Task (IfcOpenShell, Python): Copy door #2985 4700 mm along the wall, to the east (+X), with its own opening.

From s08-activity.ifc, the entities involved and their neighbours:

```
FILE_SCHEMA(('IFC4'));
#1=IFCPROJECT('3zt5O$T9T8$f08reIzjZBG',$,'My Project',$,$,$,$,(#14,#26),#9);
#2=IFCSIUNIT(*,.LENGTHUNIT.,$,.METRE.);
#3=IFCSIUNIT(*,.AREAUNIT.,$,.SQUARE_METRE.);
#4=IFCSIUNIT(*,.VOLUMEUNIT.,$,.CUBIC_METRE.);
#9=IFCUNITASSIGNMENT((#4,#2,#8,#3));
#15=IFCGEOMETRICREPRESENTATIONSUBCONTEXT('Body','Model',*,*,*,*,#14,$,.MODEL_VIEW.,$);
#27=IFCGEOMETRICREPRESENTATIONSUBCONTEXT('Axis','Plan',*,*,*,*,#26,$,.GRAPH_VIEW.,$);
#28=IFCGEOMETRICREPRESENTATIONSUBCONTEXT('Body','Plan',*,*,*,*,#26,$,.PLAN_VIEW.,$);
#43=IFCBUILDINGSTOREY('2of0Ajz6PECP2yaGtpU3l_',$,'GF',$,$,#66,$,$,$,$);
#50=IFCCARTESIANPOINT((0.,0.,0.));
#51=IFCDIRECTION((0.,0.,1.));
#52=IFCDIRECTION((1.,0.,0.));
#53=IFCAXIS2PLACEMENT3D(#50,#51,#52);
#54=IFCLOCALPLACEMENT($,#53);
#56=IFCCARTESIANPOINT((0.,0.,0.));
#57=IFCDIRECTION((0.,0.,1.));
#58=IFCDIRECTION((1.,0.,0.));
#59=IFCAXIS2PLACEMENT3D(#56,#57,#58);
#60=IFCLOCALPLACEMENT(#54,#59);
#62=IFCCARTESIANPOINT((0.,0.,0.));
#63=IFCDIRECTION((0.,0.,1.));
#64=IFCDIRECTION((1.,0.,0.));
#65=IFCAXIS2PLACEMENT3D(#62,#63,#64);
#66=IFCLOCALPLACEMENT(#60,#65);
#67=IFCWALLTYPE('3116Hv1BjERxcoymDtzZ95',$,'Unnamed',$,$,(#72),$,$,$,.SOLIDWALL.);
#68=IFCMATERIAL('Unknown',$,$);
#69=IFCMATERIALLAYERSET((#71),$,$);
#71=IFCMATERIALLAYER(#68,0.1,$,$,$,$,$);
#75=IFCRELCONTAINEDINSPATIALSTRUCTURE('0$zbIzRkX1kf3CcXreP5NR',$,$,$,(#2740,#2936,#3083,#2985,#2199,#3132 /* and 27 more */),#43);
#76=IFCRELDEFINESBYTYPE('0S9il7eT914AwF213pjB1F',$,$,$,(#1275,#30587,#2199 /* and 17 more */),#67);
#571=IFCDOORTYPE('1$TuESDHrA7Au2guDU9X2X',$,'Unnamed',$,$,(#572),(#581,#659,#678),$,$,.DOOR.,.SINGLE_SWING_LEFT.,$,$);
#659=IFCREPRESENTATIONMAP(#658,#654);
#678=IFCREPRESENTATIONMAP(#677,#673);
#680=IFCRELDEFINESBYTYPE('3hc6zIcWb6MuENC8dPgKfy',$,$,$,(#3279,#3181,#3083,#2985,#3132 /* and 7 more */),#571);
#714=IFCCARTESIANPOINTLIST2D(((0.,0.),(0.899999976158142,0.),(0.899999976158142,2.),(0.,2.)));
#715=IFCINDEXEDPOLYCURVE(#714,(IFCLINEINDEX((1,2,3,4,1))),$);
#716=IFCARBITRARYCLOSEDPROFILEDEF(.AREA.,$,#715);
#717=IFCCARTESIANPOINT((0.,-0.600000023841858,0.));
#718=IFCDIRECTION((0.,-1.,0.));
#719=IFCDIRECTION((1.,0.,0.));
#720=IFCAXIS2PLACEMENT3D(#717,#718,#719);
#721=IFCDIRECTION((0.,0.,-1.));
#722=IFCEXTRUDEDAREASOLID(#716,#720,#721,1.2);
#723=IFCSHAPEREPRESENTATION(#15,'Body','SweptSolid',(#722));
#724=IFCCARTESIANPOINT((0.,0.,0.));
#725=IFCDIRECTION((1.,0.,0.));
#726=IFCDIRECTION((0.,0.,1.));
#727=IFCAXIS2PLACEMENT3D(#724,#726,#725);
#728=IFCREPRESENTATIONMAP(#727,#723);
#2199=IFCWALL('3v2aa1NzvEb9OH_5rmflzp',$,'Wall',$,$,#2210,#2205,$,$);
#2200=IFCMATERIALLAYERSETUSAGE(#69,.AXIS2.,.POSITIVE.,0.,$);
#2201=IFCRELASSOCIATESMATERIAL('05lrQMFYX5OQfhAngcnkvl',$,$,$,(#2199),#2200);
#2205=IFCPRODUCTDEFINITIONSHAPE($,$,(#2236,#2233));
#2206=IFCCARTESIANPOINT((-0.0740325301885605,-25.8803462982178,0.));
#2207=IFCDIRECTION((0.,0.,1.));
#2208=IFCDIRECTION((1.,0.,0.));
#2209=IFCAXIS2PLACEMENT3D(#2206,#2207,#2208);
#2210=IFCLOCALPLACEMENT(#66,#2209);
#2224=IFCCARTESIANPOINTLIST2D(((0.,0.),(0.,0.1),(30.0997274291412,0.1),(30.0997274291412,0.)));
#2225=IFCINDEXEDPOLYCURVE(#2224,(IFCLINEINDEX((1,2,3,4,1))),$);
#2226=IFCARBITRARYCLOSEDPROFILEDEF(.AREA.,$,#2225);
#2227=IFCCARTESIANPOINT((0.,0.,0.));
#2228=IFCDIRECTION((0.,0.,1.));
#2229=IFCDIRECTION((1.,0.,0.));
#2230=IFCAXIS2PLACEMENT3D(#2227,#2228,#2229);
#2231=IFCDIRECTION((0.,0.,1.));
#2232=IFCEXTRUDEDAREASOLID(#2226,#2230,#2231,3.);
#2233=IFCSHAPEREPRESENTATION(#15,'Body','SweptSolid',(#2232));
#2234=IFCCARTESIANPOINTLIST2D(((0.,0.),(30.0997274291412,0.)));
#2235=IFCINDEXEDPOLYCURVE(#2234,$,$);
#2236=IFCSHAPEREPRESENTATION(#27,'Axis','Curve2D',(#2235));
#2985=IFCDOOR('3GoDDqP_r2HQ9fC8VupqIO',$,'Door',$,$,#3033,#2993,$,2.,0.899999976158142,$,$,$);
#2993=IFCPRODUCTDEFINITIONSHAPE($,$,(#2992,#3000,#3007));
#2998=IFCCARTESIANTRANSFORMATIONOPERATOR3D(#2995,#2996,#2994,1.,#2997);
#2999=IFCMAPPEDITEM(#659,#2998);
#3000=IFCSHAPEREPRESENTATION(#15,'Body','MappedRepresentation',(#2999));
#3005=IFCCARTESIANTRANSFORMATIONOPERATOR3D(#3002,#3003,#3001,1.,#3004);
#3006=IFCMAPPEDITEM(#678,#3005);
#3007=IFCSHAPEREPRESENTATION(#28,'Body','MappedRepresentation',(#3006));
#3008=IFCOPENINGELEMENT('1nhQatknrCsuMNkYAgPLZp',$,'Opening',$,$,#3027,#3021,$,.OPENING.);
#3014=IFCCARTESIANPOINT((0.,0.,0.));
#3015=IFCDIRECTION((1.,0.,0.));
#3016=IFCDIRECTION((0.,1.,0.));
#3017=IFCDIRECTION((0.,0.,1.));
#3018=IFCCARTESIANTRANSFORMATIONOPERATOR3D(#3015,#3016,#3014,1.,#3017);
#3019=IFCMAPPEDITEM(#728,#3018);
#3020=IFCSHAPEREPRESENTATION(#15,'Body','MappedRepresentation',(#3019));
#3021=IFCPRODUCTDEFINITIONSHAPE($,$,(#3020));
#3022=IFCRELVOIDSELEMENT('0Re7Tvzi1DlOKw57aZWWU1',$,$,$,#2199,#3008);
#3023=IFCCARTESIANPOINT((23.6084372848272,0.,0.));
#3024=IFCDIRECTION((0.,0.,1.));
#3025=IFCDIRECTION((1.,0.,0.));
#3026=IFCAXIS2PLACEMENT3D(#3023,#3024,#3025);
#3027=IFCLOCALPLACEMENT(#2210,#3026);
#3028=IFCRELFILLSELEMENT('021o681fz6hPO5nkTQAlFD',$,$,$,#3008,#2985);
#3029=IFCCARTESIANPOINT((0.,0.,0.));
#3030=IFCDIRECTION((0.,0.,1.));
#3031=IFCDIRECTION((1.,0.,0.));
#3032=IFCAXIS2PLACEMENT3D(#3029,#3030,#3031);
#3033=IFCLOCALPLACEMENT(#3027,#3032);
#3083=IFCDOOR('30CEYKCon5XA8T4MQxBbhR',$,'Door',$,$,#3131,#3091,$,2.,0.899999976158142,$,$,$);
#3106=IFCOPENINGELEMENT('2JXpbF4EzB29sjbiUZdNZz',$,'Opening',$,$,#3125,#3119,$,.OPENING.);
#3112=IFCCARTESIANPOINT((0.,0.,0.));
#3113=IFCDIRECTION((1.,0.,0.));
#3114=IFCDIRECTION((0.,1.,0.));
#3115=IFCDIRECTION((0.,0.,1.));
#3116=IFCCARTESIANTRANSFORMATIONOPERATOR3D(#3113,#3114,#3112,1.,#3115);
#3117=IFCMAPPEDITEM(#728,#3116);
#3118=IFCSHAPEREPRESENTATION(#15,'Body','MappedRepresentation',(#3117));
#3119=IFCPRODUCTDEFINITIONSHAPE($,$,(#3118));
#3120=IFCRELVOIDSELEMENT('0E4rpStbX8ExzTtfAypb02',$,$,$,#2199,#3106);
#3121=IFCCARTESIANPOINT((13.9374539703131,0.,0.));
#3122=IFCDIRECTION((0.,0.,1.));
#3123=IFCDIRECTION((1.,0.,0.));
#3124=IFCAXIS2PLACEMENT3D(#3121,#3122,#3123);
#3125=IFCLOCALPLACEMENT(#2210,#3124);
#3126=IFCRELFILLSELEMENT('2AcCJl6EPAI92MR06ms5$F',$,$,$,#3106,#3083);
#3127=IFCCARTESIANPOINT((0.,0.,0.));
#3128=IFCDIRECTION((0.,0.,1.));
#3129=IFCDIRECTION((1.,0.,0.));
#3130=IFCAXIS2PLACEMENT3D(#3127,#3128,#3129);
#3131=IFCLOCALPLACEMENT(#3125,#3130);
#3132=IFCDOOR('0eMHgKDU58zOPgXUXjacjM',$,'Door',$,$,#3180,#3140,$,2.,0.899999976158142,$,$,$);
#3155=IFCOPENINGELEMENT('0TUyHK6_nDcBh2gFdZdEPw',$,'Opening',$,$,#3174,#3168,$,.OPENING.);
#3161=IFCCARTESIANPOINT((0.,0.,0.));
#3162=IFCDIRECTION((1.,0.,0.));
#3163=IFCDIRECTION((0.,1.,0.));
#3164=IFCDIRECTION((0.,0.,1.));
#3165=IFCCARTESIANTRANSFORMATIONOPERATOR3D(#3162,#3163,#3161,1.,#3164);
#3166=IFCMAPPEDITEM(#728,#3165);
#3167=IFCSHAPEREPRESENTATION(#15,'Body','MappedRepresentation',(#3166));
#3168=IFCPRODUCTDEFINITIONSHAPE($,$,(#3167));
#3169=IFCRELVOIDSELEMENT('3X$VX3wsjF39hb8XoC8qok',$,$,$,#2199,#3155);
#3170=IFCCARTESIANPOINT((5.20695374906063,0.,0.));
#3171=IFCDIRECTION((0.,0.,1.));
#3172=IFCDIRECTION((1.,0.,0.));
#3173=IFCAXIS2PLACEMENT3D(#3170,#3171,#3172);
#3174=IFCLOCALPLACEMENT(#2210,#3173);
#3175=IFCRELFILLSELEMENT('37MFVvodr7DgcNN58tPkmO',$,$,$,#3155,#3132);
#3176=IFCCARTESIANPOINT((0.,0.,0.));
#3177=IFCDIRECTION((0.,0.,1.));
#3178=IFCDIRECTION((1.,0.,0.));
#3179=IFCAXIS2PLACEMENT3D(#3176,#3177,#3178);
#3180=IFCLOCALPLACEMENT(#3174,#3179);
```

```python
import ifcopenshell
import ifcopenshell.api.feature
import ifcopenshell.api.geometry
import ifcopenshell.api.root
import ifcopenshell.geom
import ifcopenshell.util.element
import ifcopenshell.util.placement
import ifcopenshell.util.shape
import ifcopenshell.util.unit

model = ifcopenshell.open("s08-activity.ifc")
unit_scale = ifcopenshell.util.unit.calculate_unit_scale(model)
settings = ifcopenshell.geom.settings()


def volume(element):
    """Net volume in cubic metres, openings subtracted."""
    shape = ifcopenshell.geom.create_shape(settings, element)
    return ifcopenshell.util.shape.get_volume(shape.geometry)


door = model.by_guid("3GoDDqP_r2HQ9fC8VupqIO")
opening = door.FillsVoids[0].RelatingOpeningElement
wall = opening.VoidsElements[0].RelatingBuildingElement
before = volume(wall)
shift = ifcopenshell.util.placement.get_local_placement(wall.ObjectPlacement)[:3, 0] * 4.7 / unit_scale

# copy_class copies the void relationship, type, container and properties, but no geometry.
new_opening = ifcopenshell.api.root.copy_class(model, product=opening)
new_opening.Representation = ifcopenshell.util.element.copy_deep(
    model, opening.Representation, exclude=["IfcGeometricRepresentationContext", "IfcRepresentationMap"]
)
new_door = ifcopenshell.api.root.copy_class(model, product=door)
new_door.Representation = ifcopenshell.util.element.copy_deep(
    model, door.Representation, exclude=["IfcGeometricRepresentationContext", "IfcRepresentationMap"]
)
ifcopenshell.api.feature.add_filling(model, opening=new_opening, element=new_door)

for old, new in ((opening, new_opening), (door, new_door)):
    matrix = ifcopenshell.util.placement.get_local_placement(old.ObjectPlacement)
    matrix[:3, 3] += shift
    ifcopenshell.api.geometry.edit_object_placement(model, product=new, matrix=matrix, is_si=False)

after = volume(wall)

print(f"wall volume {before:.3f} -> {after:.3f} m3")

model.write("s08-activity_rev.ifc")
```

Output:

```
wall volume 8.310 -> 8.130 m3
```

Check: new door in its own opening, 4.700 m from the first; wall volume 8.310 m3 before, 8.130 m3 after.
